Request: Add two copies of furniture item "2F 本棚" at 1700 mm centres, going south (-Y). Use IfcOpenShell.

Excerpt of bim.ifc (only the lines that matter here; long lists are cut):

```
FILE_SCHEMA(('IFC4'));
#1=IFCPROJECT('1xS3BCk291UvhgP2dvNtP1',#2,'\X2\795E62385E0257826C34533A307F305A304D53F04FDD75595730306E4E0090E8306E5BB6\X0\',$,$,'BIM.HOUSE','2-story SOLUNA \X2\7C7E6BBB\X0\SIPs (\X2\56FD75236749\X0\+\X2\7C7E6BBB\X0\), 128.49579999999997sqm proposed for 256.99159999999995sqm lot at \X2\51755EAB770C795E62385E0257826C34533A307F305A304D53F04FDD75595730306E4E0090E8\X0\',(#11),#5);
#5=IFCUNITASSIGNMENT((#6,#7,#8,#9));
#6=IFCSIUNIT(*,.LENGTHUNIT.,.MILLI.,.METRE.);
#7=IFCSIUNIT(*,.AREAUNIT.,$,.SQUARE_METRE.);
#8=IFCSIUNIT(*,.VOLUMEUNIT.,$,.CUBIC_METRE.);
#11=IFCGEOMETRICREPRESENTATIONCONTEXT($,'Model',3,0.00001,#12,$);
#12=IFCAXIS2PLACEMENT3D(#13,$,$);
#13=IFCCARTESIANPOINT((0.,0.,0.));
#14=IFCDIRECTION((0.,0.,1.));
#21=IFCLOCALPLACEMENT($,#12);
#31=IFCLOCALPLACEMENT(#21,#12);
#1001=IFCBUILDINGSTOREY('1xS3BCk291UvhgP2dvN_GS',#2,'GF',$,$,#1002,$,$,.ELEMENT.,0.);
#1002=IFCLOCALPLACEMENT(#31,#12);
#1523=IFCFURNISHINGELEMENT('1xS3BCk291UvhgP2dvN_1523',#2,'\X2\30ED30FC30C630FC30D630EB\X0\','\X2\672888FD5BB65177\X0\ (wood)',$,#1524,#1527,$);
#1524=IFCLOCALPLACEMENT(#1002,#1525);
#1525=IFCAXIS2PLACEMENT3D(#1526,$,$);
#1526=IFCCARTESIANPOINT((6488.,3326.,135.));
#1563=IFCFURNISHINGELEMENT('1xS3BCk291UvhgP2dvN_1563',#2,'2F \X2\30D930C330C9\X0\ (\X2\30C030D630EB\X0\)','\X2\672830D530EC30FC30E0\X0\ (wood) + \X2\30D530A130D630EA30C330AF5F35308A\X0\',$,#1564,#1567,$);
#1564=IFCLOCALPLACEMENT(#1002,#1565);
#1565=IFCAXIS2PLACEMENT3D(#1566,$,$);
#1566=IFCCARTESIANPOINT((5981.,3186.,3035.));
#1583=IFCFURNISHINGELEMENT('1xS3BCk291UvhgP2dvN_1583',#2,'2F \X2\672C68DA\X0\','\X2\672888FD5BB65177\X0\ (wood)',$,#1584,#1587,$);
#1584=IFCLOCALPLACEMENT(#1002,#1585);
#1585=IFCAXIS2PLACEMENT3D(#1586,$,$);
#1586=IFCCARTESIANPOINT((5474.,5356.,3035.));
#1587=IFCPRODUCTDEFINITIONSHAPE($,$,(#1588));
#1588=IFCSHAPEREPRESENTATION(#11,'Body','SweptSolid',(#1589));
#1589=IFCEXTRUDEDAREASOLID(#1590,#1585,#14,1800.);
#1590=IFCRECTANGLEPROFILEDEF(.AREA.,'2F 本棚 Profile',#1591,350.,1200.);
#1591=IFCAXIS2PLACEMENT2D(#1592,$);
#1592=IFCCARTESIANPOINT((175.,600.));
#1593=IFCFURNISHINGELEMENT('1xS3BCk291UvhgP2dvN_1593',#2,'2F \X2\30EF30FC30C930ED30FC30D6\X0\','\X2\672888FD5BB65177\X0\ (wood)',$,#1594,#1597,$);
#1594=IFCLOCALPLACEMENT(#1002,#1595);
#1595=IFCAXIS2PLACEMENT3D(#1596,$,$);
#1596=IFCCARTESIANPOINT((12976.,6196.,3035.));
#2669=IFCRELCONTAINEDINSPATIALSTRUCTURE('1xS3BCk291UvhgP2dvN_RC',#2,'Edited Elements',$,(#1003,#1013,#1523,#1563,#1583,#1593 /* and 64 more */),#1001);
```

```python
import numpy as np
import ifcopenshell
import ifcopenshell.api.geometry
import ifcopenshell.api.root
import ifcopenshell.util.element
import ifcopenshell.util.placement

model = ifcopenshell.open("bim.ifc")


def reuse_history(source, copy):
    """copy_class also copies each property set's owner history, people and application; keep the originals."""
    for rel in copy.IsDefinedBy:
        if rel.is_a("IfcRelDefinesByProperties") and (history := rel.RelatingPropertyDefinition.OwnerHistory):
            rel.RelatingPropertyDefinition.OwnerHistory = source.OwnerHistory
            ifcopenshell.util.element.remove_deep2(model, history)


source = model.by_id(1583)
base = ifcopenshell.util.placement.get_local_placement(source.ObjectPlacement)
step = np.array([0.0, -1.0, 0.0]) * 1700.0

for i in range(1, 3):
    copy = ifcopenshell.api.root.copy_class(model, product=source)
    copy.Representation = ifcopenshell.util.element.copy_deep(
        model, source.Representation, exclude=["IfcGeometricRepresentationContext", "IfcRepresentationMap"]
    )
    reuse_history(source, copy)
    matrix = base.copy()
    matrix[:3, 3] += i * step
    print("added at", matrix[:3, 3].round(3) + 0.0)
    ifcopenshell.api.geometry.edit_object_placement(model, product=copy, matrix=matrix, is_si=False)

model.write("bim_v2.ifc")
```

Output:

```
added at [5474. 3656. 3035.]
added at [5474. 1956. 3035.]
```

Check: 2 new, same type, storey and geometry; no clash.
